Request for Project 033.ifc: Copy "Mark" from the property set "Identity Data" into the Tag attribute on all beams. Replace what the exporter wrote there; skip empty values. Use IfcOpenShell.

First a look at what the model holds.

```python
import ifcopenshell
import ifcopenshell.util.element

model = ifcopenshell.open("Project 033.ifc")
print(model.schema)
beams = model.by_type("IfcBeam")
print(len(beams), "beams")
for e in beams[:8]:
    source = ifcopenshell.util.element.get_pset(e, "Identity Data", "Mark")
    target = e.Tag
    print(e.id(), repr(source), repr(target), sep=" | ")
```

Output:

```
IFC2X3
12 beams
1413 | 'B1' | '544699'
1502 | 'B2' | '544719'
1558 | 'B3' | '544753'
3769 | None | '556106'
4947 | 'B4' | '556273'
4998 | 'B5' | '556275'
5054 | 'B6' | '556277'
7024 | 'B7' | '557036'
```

```python
import ifcopenshell
import ifcopenshell.util.element

model = ifcopenshell.open("Project 033.ifc")

count = 0
for e in model.by_type("IfcBeam"):
    value = ifcopenshell.util.element.get_pset(e, "Identity Data", "Mark")
    current = e.Tag
    if not value or not value.strip() or current == value:
        continue
    e.Tag = value
    count += 1

print(count, "beams updated")

model.write("Project 033_v2.ifc")
```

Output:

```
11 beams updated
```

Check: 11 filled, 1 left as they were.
